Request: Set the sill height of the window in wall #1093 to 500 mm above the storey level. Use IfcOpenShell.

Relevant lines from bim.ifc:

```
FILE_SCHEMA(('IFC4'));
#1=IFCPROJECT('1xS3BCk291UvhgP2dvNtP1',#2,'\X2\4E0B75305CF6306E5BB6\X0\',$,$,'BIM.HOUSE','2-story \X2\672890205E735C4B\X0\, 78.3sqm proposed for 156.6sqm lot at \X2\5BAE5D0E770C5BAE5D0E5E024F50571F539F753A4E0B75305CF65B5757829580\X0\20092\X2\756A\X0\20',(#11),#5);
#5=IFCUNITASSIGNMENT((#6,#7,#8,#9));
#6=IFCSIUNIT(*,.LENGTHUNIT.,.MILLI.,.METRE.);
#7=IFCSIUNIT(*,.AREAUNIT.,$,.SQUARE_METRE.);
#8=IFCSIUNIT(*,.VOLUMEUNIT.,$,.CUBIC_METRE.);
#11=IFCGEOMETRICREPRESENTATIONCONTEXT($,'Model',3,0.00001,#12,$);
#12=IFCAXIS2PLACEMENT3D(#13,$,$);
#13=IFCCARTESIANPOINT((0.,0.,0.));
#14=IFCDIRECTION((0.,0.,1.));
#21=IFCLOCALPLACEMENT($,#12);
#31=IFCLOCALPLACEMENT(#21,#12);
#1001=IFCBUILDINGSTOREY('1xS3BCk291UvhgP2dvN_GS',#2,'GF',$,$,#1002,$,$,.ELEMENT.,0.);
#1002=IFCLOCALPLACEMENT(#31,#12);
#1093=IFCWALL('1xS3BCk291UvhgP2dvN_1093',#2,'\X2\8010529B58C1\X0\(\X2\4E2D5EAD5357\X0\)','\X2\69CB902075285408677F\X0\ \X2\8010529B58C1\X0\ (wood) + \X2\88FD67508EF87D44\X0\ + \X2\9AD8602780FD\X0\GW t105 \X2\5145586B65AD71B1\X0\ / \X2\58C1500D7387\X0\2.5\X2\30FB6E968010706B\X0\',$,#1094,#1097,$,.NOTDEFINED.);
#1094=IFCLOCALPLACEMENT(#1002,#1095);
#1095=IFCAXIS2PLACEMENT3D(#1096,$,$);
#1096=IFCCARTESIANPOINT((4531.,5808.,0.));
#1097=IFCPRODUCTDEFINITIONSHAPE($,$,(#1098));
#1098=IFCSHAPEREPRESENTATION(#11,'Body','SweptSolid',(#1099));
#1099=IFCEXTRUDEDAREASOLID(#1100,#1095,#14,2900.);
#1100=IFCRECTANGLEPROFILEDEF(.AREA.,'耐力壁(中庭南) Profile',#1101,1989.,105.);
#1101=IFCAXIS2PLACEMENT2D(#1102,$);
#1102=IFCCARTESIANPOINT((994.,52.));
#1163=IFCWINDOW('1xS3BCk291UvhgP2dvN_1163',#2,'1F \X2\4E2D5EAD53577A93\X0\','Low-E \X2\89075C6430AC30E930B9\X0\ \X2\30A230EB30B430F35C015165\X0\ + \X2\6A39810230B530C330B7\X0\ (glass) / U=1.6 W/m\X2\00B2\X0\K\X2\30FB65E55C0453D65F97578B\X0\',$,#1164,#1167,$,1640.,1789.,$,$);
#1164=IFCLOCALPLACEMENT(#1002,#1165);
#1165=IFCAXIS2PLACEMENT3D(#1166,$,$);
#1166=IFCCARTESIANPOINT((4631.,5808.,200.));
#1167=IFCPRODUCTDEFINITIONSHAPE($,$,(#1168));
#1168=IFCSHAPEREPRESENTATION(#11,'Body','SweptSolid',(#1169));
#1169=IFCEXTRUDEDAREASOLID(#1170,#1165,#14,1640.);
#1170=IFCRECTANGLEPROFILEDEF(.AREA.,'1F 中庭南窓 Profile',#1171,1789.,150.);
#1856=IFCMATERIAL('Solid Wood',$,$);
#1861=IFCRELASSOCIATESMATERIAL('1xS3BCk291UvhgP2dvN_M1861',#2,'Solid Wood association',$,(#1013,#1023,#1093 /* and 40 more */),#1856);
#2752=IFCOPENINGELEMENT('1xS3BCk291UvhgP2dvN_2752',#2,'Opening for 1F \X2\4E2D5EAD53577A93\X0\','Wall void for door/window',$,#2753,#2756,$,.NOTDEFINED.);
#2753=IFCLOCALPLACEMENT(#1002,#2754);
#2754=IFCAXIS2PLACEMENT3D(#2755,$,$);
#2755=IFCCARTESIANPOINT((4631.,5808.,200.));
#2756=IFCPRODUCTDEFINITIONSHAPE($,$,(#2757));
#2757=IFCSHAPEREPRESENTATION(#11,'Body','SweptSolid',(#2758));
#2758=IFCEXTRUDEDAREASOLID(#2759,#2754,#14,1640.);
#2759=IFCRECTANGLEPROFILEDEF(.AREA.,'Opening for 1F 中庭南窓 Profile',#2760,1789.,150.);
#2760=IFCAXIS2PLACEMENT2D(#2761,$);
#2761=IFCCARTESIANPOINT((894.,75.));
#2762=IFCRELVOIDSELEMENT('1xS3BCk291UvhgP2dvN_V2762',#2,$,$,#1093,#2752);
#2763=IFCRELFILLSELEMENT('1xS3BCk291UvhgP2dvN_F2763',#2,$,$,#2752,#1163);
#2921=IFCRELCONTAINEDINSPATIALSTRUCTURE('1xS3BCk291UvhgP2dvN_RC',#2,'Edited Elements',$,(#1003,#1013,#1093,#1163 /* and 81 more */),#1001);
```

```python
import numpy as np
import ifcopenshell
import ifcopenshell.api.geometry
import ifcopenshell.geom
import ifcopenshell.util.element
import ifcopenshell.util.placement
import ifcopenshell.util.shape
import ifcopenshell.util.unit

model = ifcopenshell.open("bim.ifc")
unit_scale = ifcopenshell.util.unit.calculate_unit_scale(model)

window = model.by_id(1163)
opening = window.FillsVoids[0].RelatingOpeningElement
storey = ifcopenshell.util.element.get_container(window, ifc_class="IfcBuildingStorey")
level = ifcopenshell.util.placement.get_local_placement(storey.ObjectPlacement)[2, 3]

# The opening's origin need not be at the sill, so measure its lowest point.
shape = ifcopenshell.geom.create_shape(ifcopenshell.geom.settings(), opening)
bottom = ifcopenshell.util.shape.get_shape_bottom_elevation(shape, shape.geometry) / unit_scale
dz = level + 500.0 - bottom

shift = np.array([0.0, 0.0, dz])
# The window is not placed relative to its opening, so move both.
for product in (opening, window):
    matrix = ifcopenshell.util.placement.get_local_placement(product.ObjectPlacement)
    matrix[:3, 3] += shift
    ifcopenshell.api.geometry.edit_object_placement(model, product=product, matrix=matrix, is_si=False)

print(f"moved by {dz * unit_scale:+.3f} m")

model.write("bim_edited.ifc")
```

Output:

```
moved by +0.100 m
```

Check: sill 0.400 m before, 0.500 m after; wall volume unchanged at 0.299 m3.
